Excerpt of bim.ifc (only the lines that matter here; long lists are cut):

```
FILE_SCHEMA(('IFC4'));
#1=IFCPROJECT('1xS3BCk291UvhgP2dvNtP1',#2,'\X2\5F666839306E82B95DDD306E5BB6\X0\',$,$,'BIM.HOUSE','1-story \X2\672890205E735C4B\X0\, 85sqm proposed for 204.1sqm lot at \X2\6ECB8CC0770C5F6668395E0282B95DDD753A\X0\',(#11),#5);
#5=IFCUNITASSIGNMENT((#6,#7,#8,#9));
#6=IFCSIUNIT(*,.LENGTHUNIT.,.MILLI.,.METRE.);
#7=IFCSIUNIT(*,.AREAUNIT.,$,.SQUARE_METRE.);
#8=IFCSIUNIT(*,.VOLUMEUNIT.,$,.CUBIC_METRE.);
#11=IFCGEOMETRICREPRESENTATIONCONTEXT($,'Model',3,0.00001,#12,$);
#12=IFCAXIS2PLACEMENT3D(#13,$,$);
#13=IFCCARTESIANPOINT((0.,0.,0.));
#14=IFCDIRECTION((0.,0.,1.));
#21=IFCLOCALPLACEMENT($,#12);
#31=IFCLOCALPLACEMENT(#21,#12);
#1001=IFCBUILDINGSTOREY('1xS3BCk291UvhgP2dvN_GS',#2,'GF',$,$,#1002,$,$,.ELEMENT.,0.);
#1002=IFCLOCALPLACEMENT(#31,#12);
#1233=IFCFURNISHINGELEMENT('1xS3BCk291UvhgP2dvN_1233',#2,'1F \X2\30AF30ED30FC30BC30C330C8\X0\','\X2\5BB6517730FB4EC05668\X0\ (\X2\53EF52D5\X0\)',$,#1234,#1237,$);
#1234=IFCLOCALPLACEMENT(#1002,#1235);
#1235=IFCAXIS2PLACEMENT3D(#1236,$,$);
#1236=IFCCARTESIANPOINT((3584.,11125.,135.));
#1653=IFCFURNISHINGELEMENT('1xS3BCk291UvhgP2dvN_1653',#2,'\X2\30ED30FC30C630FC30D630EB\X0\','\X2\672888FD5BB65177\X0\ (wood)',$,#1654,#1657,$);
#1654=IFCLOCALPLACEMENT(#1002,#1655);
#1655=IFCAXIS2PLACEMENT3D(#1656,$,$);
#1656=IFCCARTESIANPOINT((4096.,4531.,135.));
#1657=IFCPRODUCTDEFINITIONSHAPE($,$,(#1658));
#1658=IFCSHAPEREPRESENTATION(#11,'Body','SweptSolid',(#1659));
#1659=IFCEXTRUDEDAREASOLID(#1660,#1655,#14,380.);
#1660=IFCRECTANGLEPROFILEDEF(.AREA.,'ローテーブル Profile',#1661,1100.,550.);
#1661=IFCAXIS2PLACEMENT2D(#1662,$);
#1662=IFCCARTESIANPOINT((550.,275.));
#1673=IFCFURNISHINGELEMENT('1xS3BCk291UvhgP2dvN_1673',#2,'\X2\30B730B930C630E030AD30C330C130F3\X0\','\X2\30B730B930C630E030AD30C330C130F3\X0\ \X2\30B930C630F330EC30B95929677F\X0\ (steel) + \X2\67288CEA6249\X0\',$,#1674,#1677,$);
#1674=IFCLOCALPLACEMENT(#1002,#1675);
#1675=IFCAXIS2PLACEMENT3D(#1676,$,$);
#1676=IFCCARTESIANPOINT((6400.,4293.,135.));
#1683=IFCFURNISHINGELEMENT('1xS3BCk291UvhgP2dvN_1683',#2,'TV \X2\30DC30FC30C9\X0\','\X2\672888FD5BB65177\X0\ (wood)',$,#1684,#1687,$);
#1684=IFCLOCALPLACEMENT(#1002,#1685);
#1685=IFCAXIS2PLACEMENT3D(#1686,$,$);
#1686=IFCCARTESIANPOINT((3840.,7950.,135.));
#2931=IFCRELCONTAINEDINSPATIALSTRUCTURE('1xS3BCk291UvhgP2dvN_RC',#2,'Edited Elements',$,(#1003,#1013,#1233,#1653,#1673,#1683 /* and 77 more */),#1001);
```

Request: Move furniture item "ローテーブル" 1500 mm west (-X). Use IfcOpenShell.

```python
import ifcopenshell
import ifcopenshell.api.geometry
import ifcopenshell.util.placement
import ifcopenshell.util.unit

model = ifcopenshell.open("bim.ifc")
unit_scale = ifcopenshell.util.unit.calculate_unit_scale(model)

item = model.by_guid("1xS3BCk291UvhgP2dvN_1653")
matrix = ifcopenshell.util.placement.get_local_placement(item.ObjectPlacement)
matrix[0, 3] -= 1.5 / unit_scale
ifcopenshell.api.geometry.edit_object_placement(model, product=item, matrix=matrix, is_si=False)

print(ifcopenshell.util.placement.get_local_placement(item.ObjectPlacement).round(3) + 0.0)

model.write("bim_v2.ifc")
```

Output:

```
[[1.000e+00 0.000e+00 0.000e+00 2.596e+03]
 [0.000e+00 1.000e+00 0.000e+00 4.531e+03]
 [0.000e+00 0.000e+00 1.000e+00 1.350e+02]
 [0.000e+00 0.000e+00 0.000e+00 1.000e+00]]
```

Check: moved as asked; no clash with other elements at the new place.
